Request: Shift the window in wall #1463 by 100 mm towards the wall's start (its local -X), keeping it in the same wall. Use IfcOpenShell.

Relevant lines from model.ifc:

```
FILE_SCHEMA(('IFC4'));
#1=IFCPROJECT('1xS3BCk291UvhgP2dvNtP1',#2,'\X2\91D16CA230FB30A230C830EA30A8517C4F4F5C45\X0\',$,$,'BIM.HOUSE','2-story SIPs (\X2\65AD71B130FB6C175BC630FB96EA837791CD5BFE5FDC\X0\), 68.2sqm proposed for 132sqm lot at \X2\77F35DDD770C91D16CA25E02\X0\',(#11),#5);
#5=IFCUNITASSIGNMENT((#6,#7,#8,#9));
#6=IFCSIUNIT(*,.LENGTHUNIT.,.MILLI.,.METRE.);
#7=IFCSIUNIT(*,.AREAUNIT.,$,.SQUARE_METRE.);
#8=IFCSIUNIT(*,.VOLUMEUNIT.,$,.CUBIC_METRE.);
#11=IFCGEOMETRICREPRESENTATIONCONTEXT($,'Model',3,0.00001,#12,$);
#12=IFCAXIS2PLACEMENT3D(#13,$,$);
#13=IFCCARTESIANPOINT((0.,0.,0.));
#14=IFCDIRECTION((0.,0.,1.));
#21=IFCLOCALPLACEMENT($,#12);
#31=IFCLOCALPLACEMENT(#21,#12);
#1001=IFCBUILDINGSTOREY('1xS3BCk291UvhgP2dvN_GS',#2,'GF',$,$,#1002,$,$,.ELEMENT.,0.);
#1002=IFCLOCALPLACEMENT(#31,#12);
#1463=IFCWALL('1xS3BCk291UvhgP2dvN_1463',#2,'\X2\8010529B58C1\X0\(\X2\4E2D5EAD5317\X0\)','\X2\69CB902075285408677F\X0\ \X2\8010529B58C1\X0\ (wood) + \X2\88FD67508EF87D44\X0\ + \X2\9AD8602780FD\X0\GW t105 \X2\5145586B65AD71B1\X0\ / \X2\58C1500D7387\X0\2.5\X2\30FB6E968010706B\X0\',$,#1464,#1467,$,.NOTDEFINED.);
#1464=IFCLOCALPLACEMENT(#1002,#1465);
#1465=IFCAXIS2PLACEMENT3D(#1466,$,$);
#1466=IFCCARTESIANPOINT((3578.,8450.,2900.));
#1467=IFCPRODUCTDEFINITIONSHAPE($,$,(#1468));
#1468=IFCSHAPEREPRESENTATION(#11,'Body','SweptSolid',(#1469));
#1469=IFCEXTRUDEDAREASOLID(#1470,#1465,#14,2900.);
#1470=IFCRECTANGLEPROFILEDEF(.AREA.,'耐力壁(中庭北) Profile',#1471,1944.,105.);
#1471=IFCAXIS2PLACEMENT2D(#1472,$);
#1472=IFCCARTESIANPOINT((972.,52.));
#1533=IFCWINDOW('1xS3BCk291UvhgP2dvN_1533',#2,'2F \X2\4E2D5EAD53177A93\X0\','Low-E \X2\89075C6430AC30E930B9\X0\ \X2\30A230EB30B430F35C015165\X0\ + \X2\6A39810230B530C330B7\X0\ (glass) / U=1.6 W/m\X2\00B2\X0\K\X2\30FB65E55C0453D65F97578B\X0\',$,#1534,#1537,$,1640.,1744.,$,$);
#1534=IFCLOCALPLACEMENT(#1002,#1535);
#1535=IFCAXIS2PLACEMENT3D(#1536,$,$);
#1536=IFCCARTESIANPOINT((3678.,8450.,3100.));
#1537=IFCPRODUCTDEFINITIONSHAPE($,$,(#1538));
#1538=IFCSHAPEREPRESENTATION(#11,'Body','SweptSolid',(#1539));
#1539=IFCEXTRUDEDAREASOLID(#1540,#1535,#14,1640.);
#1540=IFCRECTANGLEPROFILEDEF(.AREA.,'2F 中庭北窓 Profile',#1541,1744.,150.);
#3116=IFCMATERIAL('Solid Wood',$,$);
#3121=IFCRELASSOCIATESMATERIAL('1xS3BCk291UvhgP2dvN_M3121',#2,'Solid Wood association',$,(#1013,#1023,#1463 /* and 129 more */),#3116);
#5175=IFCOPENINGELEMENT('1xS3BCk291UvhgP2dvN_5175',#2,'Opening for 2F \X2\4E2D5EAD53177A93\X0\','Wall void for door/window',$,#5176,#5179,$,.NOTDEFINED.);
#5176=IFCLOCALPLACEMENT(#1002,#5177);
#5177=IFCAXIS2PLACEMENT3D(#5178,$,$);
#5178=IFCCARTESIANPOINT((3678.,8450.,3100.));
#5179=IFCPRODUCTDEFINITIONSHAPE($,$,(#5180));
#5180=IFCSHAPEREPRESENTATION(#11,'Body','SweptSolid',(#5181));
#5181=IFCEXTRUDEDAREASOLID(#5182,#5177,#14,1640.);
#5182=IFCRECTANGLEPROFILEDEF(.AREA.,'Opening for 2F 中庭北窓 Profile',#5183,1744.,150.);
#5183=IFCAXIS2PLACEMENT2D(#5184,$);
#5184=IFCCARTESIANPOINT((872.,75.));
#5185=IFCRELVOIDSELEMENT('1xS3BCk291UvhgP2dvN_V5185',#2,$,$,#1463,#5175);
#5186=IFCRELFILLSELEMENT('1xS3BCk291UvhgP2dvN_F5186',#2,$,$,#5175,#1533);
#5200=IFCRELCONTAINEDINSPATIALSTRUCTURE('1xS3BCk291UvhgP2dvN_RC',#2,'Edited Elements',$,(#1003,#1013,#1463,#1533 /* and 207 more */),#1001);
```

```python
import ifcopenshell
import ifcopenshell.api.geometry
import ifcopenshell.util.placement
import ifcopenshell.util.unit

model = ifcopenshell.open("model.ifc")
unit_scale = ifcopenshell.util.unit.calculate_unit_scale(model)

window = model.by_guid("1xS3BCk291UvhgP2dvN_1533")
opening = window.FillsVoids[0].RelatingOpeningElement
wall = opening.VoidsElements[0].RelatingBuildingElement

wall_matrix = ifcopenshell.util.placement.get_local_placement(wall.ObjectPlacement)
shift = wall_matrix[:3, 0] * -0.1 / unit_scale
before = ifcopenshell.util.placement.get_local_placement(window.ObjectPlacement)[:3, 3].copy()

# The window is not placed relative to its opening, so move both.
for product in (opening, window):
    matrix = ifcopenshell.util.placement.get_local_placement(product.ObjectPlacement)
    matrix[:3, 3] += shift
    ifcopenshell.api.geometry.edit_object_placement(model, product=product, matrix=matrix, is_si=False)

after = ifcopenshell.util.placement.get_local_placement(window.ObjectPlacement)[:3, 3]
print("window moved by", (after - before).round(3) + 0.0)

model.write("model_edited.ifc")
```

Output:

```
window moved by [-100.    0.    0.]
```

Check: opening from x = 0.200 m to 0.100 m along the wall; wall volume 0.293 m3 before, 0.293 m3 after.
